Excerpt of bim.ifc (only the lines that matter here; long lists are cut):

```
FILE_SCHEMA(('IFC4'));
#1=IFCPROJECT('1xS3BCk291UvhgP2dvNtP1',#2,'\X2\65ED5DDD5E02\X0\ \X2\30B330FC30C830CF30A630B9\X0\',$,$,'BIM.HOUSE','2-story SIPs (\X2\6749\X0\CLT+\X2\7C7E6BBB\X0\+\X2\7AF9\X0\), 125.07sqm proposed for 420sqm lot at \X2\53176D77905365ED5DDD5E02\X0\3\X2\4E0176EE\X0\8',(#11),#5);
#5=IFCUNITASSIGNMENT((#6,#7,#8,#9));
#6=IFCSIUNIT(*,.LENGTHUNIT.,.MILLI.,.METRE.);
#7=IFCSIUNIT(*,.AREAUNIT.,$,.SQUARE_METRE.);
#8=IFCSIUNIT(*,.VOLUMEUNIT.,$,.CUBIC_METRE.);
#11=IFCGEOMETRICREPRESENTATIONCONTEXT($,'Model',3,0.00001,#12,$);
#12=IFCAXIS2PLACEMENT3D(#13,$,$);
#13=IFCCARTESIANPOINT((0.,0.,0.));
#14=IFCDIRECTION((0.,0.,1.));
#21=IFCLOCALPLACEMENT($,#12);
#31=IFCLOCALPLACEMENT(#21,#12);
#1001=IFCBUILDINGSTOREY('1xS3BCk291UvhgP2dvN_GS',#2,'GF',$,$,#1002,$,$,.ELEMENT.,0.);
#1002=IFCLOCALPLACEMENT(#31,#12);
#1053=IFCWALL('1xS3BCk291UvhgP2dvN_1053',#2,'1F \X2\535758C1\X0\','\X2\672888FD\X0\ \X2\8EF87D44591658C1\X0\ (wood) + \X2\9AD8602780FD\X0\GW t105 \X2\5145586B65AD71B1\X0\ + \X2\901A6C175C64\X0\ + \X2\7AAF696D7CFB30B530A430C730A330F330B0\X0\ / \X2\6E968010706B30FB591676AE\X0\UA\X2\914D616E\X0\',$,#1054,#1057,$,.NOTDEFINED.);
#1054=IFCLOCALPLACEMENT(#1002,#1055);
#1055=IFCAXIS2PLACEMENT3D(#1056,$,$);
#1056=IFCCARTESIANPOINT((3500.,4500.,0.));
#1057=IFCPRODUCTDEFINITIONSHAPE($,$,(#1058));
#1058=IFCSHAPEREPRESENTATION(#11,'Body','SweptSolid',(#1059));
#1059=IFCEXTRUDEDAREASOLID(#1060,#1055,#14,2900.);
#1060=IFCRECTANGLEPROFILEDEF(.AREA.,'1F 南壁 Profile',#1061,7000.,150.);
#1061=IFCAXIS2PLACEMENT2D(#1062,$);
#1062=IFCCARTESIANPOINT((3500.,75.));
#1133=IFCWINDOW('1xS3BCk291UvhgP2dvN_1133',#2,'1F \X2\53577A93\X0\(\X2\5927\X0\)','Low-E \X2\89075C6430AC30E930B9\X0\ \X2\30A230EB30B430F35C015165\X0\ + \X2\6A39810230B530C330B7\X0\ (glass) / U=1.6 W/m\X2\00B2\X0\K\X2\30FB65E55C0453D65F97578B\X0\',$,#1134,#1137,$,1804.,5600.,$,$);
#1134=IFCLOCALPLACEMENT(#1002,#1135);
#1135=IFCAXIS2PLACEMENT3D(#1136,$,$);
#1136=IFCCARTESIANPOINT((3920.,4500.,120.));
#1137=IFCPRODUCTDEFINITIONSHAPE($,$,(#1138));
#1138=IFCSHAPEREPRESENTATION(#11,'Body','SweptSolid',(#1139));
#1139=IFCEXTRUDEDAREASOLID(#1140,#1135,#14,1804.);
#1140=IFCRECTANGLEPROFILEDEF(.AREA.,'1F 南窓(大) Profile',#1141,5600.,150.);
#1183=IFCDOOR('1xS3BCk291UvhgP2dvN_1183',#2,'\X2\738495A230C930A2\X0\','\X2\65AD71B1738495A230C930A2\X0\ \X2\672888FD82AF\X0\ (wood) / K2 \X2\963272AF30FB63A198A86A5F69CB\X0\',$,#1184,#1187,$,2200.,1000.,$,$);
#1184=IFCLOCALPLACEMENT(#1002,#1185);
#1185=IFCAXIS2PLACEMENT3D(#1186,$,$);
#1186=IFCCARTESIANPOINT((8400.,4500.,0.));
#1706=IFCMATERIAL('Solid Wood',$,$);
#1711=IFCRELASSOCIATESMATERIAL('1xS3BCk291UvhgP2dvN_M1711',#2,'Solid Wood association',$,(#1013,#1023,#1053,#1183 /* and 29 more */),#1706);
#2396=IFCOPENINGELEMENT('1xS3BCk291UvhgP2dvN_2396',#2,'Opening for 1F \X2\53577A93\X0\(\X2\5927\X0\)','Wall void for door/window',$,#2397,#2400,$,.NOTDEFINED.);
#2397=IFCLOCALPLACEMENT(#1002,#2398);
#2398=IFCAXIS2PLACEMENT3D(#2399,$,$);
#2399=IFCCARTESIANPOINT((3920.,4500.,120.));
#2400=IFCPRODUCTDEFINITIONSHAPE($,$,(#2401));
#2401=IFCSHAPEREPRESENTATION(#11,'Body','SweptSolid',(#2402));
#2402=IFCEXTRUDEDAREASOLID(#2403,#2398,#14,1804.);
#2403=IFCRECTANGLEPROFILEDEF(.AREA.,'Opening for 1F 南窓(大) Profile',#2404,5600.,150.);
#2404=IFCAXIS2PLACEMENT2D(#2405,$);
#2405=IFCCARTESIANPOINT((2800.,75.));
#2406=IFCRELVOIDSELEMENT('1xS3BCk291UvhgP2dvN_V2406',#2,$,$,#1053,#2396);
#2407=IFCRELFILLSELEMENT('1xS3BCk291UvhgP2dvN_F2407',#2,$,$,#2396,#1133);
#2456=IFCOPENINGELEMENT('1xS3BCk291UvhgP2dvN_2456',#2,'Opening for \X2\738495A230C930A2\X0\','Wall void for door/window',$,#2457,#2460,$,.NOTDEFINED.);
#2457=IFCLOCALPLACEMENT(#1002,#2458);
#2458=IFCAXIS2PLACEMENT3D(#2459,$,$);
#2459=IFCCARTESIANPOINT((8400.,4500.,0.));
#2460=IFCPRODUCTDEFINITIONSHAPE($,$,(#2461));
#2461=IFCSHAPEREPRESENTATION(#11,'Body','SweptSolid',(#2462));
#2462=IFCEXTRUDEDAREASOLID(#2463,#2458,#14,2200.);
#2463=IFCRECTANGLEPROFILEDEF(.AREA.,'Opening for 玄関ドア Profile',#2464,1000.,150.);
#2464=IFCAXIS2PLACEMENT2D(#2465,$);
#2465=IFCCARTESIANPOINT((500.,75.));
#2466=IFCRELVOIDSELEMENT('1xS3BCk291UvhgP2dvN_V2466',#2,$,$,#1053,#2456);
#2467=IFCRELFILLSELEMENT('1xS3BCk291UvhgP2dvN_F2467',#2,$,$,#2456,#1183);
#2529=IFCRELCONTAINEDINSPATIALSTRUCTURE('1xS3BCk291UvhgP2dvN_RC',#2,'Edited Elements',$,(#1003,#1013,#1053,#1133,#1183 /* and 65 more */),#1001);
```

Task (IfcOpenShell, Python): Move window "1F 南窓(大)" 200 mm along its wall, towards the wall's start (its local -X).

```python
import ifcopenshell
import ifcopenshell.api.geometry
import ifcopenshell.util.placement

model = ifcopenshell.open("bim.ifc")

window = model.by_guid("1xS3BCk291UvhgP2dvN_1133")
opening = window.FillsVoids[0].RelatingOpeningElement
wall = opening.VoidsElements[0].RelatingBuildingElement

wall_matrix = ifcopenshell.util.placement.get_local_placement(wall.ObjectPlacement)
shift = wall_matrix[:3, 0] * -200.0
before = ifcopenshell.util.placement.get_local_placement(window.ObjectPlacement)[:3, 3].copy()

# The window is not placed relative to its opening, so move both.
for product in (opening, window):
    matrix = ifcopenshell.util.placement.get_local_placement(product.ObjectPlacement)
    matrix[:3, 3] += shift
    ifcopenshell.api.geometry.edit_object_placement(model, product=product, matrix=matrix, is_si=False)

after = ifcopenshell.util.placement.get_local_placement(window.ObjectPlacement)[:3, 3]
print("window moved by", (after - before).round(3) + 0.0)

model.write("bim-out.ifc")
```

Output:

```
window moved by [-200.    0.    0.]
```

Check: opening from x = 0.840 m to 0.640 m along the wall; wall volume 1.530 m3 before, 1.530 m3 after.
